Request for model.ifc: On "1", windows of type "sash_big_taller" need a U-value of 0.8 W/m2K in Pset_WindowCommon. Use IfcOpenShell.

First a look at what the model holds.

```python
import ifcopenshell
import ifcopenshell.util.element

model = ifcopenshell.open("model.ifc")
print(model.schema)
storey = next(s for s in model.by_type("IfcBuildingStorey") if s.Name == "1")
windows = [e for e in ifcopenshell.util.element.get_decomposition(storey) if e.is_a("IfcWindow")]
seen = {}
for e in windows:
    element_type = ifcopenshell.util.element.get_type(e)
    key = (element_type.Name if element_type != e and element_type else None, ifcopenshell.util.element.get_pset(e, "Pset_WindowCommon", "ThermalTransmittance"))
    seen[key] = seen.get(key, 0) + 1
for (name, value), count in sorted(seen.items(), key=str):
    print(count, "x", name, "|", value)
```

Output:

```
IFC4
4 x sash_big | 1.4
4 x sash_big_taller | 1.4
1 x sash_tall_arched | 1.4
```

```python
import ifcopenshell
import ifcopenshell.api.pset
import ifcopenshell.util.element

model = ifcopenshell.open("model.ifc")

storey = next(s for s in model.by_type("IfcBuildingStorey") if s.Name == "1")
windows = [e for e in ifcopenshell.util.element.get_decomposition(storey) if e.is_a("IfcWindow")]

count = 0
for e in windows:
    element_type = ifcopenshell.util.element.get_type(e)
    if element_type in (None, e) or element_type.Name != "sash_big_taller":
        continue
    # add_pset returns the element's existing set when there is one.
    pset = ifcopenshell.api.pset.add_pset(model, product=e, name="Pset_WindowCommon")
    ifcopenshell.api.pset.edit_pset(model, pset=pset, properties={"ThermalTransmittance": 0.8})
    count += 1

print(count, "windows updated")

model.write("model_v2.ifc")
```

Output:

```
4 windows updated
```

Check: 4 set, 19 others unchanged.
